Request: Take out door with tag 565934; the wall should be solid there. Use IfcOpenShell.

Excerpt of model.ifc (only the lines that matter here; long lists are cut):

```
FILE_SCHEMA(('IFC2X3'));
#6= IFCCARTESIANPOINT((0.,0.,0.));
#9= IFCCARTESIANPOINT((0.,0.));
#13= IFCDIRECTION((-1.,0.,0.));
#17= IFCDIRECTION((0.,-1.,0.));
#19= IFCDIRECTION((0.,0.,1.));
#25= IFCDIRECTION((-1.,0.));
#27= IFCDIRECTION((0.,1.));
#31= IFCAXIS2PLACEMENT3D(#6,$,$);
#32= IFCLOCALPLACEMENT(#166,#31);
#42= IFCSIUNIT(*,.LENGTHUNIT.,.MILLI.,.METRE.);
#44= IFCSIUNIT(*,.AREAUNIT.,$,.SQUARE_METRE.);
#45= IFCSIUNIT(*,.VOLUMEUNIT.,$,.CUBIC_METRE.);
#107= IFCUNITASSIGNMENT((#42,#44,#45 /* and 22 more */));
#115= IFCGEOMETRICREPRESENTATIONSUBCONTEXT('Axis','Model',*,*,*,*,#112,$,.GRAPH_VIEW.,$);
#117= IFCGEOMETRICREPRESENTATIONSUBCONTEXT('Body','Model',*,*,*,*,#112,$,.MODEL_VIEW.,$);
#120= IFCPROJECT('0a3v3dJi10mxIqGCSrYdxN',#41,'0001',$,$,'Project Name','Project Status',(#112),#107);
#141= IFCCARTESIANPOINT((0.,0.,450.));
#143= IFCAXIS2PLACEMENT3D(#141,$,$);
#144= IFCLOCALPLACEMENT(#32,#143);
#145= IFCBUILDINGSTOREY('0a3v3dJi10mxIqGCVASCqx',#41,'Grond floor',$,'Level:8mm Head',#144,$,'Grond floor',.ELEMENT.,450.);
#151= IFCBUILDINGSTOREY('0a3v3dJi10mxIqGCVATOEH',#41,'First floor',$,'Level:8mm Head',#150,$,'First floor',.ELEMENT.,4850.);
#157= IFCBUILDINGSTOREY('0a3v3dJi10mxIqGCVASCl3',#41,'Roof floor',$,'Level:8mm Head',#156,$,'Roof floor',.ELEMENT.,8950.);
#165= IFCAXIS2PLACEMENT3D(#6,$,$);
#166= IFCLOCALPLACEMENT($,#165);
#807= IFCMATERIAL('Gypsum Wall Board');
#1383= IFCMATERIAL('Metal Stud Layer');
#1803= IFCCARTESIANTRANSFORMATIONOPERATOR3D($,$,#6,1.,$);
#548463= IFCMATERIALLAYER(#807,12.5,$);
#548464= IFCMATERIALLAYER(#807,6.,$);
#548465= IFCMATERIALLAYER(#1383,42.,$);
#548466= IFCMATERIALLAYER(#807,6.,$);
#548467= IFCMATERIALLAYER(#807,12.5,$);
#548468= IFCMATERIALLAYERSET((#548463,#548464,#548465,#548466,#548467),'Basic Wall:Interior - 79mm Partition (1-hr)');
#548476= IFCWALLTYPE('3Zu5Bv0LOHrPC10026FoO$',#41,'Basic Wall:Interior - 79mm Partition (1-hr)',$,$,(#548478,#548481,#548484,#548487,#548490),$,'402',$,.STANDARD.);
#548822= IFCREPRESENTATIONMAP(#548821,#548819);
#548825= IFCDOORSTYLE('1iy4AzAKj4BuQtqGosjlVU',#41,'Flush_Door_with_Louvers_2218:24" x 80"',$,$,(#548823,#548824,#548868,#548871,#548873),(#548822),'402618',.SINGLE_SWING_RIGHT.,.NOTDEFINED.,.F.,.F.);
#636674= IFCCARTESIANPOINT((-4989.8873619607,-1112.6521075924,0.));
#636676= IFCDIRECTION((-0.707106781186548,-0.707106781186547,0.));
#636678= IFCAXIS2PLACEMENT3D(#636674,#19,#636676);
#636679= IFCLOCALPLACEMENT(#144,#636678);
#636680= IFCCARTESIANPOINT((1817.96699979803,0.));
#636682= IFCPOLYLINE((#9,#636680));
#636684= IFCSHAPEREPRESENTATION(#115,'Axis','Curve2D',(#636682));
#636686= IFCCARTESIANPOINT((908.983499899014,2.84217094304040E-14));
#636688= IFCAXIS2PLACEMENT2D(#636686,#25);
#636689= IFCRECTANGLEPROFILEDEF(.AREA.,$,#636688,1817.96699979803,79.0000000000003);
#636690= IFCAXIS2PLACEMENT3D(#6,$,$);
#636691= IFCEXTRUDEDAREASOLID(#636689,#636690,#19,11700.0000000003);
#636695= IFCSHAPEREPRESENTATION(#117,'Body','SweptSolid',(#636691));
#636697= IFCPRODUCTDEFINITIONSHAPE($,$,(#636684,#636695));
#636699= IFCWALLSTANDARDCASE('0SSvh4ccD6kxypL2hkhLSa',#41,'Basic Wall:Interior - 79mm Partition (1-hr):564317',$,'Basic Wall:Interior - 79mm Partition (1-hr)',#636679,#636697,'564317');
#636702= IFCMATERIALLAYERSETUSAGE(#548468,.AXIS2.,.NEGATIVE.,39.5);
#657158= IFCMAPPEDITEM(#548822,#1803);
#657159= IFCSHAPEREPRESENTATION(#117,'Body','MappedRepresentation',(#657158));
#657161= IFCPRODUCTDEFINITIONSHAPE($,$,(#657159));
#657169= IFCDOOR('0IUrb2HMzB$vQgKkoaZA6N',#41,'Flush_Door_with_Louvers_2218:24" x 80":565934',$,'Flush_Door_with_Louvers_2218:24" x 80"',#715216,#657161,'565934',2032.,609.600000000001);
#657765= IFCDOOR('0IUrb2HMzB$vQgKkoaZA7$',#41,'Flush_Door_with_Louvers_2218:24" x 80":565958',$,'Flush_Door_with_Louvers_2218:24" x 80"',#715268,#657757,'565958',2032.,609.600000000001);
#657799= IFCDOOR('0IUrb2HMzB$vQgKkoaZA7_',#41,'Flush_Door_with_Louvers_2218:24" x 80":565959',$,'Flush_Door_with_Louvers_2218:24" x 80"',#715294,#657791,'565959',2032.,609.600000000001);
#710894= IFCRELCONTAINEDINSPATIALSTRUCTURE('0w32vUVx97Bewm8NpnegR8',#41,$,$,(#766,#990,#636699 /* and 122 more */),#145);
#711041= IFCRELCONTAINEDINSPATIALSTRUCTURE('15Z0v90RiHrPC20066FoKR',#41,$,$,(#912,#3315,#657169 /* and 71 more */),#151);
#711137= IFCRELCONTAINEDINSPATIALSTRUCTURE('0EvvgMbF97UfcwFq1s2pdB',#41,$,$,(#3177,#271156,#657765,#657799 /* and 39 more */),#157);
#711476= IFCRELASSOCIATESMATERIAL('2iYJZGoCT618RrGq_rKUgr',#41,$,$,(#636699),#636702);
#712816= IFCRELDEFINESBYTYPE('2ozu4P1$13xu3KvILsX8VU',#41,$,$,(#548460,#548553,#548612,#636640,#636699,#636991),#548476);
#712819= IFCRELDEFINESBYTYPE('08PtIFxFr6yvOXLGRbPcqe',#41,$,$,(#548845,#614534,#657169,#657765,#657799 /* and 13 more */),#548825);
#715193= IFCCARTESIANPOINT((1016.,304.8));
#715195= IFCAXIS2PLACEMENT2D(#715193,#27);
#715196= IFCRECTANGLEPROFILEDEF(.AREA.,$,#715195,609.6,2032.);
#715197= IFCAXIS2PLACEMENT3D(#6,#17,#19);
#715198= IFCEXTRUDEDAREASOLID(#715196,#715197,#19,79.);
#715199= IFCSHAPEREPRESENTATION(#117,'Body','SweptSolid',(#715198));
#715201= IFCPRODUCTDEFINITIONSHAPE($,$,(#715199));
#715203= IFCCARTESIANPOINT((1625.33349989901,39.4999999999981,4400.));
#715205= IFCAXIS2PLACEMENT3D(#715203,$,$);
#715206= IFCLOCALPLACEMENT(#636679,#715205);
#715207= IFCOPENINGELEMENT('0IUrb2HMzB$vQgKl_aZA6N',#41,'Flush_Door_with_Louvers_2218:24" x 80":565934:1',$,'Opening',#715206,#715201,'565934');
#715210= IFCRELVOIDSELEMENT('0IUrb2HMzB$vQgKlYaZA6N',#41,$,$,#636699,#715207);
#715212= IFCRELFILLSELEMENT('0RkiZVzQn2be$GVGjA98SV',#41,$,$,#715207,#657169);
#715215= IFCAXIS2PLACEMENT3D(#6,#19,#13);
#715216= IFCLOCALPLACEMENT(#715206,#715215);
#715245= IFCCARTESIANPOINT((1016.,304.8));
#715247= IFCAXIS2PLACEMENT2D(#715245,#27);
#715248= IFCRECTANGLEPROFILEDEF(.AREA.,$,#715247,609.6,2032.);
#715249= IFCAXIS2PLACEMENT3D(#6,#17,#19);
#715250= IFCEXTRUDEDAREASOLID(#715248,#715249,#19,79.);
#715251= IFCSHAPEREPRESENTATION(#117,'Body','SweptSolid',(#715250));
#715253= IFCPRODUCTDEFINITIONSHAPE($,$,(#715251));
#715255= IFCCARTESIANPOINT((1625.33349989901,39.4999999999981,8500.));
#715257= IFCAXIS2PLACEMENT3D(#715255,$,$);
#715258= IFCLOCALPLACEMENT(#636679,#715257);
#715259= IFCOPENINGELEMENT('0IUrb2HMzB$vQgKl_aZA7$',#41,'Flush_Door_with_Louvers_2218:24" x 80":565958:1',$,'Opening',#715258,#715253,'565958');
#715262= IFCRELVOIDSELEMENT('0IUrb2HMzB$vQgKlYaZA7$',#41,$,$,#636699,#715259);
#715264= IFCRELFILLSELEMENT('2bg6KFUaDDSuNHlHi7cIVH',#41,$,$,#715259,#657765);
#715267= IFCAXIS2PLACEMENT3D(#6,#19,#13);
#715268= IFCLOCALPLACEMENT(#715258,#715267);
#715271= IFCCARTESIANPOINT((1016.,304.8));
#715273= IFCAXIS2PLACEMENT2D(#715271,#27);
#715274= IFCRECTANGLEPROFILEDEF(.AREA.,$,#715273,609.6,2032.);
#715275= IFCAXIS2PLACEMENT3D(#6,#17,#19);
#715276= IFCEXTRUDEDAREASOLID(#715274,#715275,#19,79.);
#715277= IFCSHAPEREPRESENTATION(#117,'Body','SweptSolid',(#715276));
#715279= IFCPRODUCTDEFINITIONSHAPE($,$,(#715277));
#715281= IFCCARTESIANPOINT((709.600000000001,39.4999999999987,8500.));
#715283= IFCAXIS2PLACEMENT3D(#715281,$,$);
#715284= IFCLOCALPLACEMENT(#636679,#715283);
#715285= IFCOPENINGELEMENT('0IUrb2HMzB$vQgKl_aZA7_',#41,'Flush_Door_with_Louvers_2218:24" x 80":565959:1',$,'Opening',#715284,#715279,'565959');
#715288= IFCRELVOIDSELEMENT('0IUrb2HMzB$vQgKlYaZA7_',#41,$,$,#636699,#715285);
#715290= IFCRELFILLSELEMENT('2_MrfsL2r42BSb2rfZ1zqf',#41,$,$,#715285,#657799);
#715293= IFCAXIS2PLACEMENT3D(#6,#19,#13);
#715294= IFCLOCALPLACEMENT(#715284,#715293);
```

```python
import ifcopenshell
import ifcopenshell.api.feature
import ifcopenshell.api.root
import ifcopenshell.geom
import ifcopenshell.util.shape

model = ifcopenshell.open("model.ifc")
settings = ifcopenshell.geom.settings()


def volume(element):
    """Net volume in cubic metres, openings subtracted."""
    shape = ifcopenshell.geom.create_shape(settings, element)
    return ifcopenshell.util.shape.get_volume(shape.geometry)


door = model.by_guid("0IUrb2HMzB$vQgKkoaZA6N")
opening = door.FillsVoids[0].RelatingOpeningElement
wall = opening.VoidsElements[0].RelatingBuildingElement
before = volume(wall)

ifcopenshell.api.root.remove_product(model, product=door)
ifcopenshell.api.feature.remove_feature(model, feature=opening)

after = volume(wall)

print(f"wall volume {before:.3f} -> {after:.3f} m3")

model.write("model_rev.ifc")
```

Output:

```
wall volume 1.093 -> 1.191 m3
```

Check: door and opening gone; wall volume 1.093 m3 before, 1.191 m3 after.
